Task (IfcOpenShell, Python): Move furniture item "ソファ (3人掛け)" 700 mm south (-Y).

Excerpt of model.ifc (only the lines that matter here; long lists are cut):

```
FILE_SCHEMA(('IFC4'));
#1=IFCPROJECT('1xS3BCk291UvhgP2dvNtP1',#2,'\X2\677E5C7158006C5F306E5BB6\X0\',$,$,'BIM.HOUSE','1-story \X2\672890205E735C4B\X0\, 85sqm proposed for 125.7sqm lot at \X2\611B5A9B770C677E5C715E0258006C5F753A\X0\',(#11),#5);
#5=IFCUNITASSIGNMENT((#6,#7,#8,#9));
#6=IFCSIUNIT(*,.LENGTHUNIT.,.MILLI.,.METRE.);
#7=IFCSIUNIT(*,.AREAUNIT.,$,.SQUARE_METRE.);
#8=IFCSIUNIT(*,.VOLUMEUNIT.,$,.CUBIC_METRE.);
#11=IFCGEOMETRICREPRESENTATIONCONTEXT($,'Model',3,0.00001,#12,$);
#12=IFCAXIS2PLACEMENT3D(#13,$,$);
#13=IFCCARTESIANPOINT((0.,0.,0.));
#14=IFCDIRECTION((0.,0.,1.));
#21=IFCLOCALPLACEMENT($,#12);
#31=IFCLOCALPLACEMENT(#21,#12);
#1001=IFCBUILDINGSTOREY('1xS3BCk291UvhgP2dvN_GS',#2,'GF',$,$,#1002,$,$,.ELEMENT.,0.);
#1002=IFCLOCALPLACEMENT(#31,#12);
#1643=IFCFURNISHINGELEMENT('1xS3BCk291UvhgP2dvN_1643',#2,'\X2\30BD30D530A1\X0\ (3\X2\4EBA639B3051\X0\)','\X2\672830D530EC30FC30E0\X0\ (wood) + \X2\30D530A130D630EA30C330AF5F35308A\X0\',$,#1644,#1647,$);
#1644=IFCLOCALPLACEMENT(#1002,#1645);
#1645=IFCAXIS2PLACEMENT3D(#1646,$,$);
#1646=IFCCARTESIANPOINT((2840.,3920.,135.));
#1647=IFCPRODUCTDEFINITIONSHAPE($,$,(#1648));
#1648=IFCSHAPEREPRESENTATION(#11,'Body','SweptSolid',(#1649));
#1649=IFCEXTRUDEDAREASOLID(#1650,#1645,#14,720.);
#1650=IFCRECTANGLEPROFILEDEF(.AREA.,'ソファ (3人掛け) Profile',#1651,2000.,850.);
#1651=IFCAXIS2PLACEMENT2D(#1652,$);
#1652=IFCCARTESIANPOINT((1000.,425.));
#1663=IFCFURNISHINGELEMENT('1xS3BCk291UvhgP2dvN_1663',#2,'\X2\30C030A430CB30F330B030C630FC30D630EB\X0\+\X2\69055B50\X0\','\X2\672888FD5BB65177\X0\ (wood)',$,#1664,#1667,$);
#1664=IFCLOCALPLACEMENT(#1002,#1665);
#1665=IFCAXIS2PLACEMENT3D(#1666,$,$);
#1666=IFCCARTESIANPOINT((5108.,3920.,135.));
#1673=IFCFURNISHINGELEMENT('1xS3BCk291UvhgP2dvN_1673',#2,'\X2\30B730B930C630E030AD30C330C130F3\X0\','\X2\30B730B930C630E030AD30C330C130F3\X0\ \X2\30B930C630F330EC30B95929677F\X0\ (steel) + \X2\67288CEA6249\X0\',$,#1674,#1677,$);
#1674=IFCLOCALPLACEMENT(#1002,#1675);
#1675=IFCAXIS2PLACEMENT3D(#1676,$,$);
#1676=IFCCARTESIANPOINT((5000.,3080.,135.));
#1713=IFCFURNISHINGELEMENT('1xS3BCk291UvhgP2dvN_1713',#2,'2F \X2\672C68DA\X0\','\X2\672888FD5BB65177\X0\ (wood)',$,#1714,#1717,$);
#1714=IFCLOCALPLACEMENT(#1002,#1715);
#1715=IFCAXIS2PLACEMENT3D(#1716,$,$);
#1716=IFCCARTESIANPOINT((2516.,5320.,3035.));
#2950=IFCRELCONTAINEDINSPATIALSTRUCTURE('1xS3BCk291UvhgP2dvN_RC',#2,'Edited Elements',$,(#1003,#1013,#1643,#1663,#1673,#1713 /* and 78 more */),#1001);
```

```python
import ifcopenshell
import ifcopenshell.api.geometry
import ifcopenshell.util.placement
import ifcopenshell.util.unit

model = ifcopenshell.open("model.ifc")
unit_scale = ifcopenshell.util.unit.calculate_unit_scale(model)

item = model.by_guid("1xS3BCk291UvhgP2dvN_1643")
matrix = ifcopenshell.util.placement.get_local_placement(item.ObjectPlacement)
matrix[1, 3] -= 0.7 / unit_scale
ifcopenshell.api.geometry.edit_object_placement(model, product=item, matrix=matrix, is_si=False)

print(ifcopenshell.util.placement.get_local_placement(item.ObjectPlacement).round(3) + 0.0)

model.write("model_v2.ifc")
```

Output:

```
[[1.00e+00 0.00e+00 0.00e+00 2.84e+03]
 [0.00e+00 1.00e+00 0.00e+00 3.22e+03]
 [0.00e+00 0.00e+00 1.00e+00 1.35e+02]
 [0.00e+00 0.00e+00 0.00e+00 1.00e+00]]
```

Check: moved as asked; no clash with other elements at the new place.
